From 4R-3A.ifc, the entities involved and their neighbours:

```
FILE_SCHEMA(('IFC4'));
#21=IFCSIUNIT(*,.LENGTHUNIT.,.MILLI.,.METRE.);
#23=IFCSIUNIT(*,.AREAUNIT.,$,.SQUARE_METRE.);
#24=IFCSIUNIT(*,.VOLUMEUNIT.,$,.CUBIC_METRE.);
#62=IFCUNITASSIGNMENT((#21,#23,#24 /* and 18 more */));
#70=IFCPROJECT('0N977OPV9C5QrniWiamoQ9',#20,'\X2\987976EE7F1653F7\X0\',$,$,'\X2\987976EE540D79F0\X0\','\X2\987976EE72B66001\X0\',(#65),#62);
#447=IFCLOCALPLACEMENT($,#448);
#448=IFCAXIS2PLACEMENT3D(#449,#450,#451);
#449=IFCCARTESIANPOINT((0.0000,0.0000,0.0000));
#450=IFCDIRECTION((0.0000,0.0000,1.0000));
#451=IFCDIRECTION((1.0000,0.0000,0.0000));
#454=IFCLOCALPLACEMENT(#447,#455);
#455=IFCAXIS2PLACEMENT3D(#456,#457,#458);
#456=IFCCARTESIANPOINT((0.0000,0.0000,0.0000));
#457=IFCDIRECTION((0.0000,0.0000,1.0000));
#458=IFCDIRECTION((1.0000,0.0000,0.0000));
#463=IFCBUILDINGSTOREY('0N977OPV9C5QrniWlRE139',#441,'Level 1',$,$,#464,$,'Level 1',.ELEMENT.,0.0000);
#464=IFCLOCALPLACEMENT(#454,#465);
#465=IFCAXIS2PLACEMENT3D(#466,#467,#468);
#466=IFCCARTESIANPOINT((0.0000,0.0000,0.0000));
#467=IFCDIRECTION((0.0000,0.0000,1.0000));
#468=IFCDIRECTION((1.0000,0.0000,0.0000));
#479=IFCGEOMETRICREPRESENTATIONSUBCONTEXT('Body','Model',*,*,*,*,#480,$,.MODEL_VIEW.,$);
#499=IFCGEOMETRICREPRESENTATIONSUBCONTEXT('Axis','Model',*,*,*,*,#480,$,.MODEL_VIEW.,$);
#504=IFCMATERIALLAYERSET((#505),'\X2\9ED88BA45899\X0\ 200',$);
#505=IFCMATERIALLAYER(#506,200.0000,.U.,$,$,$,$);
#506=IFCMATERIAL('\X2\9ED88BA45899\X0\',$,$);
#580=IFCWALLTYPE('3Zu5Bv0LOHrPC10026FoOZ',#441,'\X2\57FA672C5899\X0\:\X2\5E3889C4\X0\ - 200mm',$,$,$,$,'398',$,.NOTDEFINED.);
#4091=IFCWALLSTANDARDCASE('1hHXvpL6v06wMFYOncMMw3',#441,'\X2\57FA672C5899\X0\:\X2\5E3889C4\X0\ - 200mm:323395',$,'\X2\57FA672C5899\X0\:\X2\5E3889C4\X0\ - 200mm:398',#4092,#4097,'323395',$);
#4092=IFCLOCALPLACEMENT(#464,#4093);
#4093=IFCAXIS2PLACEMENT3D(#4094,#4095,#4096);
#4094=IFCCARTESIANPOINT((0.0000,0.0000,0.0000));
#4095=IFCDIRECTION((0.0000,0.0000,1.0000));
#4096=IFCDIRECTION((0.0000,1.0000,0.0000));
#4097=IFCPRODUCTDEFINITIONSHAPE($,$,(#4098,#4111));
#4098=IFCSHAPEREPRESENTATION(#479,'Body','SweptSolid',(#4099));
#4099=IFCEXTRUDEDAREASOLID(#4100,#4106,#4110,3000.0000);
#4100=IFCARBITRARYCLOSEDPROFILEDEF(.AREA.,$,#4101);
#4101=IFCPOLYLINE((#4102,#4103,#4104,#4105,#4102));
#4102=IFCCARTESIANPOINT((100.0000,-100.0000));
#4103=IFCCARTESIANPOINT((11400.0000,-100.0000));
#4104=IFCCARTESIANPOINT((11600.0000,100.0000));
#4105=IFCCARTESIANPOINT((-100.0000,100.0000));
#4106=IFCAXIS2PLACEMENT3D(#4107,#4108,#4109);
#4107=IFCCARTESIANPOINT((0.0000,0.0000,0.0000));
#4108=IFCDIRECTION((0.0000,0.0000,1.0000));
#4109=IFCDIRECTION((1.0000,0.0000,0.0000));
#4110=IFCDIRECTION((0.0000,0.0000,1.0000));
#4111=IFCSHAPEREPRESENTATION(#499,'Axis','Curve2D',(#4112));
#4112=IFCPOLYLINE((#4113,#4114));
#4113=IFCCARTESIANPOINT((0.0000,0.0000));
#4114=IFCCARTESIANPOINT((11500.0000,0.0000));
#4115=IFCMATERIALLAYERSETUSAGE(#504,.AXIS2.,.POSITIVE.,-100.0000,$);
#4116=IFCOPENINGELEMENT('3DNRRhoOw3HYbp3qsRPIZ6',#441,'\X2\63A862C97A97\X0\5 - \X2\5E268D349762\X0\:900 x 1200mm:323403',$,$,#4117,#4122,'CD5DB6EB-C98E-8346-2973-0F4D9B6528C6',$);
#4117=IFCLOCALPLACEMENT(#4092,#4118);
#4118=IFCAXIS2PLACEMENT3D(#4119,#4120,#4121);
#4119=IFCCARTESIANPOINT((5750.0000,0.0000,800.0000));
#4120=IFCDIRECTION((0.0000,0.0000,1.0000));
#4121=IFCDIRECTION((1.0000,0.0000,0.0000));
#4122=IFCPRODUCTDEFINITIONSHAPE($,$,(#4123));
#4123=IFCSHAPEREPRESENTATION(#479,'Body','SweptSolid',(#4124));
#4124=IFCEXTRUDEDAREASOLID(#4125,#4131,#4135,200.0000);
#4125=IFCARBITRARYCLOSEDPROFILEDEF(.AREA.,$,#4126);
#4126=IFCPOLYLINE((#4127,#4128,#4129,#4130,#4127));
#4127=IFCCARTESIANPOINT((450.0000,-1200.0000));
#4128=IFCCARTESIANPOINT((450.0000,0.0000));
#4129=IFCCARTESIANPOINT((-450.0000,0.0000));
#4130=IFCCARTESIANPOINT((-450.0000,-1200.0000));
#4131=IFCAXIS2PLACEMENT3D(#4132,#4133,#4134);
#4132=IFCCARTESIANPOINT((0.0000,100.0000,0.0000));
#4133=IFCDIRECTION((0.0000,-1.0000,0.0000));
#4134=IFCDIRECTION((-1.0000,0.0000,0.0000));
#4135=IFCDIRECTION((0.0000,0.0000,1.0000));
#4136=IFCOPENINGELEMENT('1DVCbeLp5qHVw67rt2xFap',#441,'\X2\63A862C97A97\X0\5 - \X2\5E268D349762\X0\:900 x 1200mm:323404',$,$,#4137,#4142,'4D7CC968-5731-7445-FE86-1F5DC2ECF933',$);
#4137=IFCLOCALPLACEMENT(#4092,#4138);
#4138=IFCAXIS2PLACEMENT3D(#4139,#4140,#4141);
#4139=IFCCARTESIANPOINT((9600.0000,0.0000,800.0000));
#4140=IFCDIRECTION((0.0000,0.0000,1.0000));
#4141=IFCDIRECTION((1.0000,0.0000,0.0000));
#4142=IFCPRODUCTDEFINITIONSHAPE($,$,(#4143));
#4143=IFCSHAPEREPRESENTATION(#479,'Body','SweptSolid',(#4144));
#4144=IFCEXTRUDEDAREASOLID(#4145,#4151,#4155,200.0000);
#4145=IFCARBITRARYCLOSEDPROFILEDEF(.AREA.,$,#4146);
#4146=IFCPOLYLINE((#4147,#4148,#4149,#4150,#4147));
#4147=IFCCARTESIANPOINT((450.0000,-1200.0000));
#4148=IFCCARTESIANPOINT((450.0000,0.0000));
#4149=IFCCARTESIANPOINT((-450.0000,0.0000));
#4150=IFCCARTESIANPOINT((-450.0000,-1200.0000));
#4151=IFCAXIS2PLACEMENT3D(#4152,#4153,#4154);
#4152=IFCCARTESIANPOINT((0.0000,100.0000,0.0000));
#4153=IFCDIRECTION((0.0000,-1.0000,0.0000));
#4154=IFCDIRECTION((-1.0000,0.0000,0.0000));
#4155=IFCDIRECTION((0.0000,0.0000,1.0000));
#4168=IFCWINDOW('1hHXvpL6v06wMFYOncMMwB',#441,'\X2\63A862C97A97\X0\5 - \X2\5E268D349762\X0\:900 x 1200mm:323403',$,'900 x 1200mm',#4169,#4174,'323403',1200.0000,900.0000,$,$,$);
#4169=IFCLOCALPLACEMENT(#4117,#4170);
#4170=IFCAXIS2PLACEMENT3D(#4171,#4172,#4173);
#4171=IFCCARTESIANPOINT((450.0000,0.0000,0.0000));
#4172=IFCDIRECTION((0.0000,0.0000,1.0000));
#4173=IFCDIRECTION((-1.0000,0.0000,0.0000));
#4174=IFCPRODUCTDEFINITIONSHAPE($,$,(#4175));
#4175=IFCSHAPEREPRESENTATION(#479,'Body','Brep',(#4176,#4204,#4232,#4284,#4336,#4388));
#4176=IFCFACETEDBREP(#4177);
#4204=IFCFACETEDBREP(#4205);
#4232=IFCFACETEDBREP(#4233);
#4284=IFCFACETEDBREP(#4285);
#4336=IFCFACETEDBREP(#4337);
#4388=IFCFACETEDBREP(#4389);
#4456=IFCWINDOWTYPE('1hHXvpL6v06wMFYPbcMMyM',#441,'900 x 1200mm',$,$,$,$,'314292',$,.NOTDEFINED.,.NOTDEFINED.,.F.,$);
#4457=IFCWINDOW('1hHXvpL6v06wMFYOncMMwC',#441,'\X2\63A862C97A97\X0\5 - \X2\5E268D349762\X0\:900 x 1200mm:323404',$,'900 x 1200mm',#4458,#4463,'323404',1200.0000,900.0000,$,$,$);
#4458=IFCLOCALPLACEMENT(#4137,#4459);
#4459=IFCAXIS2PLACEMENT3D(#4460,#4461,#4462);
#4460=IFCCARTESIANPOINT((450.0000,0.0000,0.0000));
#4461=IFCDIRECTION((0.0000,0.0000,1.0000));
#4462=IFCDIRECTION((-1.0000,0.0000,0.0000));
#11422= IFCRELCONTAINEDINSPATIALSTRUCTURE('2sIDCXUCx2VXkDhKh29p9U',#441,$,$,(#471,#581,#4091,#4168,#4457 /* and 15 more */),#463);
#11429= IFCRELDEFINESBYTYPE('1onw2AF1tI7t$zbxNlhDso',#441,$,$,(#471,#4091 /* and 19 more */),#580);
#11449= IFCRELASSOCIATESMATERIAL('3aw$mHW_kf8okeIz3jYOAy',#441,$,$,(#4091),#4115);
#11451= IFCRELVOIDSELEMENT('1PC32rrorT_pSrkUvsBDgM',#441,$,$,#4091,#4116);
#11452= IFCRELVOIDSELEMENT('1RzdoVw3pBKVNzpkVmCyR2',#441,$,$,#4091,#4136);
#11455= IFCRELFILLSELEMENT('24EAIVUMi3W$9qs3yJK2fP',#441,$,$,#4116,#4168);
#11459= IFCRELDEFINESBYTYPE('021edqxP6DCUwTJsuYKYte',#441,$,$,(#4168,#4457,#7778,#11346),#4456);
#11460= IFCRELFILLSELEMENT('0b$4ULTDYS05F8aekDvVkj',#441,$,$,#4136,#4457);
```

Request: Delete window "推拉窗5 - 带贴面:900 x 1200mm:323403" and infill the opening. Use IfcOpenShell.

```python
import ifcopenshell
import ifcopenshell.api.feature
import ifcopenshell.api.root
import ifcopenshell.geom
import ifcopenshell.util.shape

model = ifcopenshell.open("4R-3A.ifc")
settings = ifcopenshell.geom.settings()


def volume(element):
    """Net volume in cubic metres, openings subtracted."""
    shape = ifcopenshell.geom.create_shape(settings, element)
    return ifcopenshell.util.shape.get_volume(shape.geometry)


window = model.by_guid("1hHXvpL6v06wMFYOncMMwB")
opening = window.FillsVoids[0].RelatingOpeningElement
wall = opening.VoidsElements[0].RelatingBuildingElement
before = volume(wall)

ifcopenshell.api.root.remove_product(model, product=window)
ifcopenshell.api.feature.remove_feature(model, feature=opening)

after = volume(wall)

print(f"wall volume {before:.3f} -> {after:.3f} m3")

model.write("4R-3A_updated.ifc")
```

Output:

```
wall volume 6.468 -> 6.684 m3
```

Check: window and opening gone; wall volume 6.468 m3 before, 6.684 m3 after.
